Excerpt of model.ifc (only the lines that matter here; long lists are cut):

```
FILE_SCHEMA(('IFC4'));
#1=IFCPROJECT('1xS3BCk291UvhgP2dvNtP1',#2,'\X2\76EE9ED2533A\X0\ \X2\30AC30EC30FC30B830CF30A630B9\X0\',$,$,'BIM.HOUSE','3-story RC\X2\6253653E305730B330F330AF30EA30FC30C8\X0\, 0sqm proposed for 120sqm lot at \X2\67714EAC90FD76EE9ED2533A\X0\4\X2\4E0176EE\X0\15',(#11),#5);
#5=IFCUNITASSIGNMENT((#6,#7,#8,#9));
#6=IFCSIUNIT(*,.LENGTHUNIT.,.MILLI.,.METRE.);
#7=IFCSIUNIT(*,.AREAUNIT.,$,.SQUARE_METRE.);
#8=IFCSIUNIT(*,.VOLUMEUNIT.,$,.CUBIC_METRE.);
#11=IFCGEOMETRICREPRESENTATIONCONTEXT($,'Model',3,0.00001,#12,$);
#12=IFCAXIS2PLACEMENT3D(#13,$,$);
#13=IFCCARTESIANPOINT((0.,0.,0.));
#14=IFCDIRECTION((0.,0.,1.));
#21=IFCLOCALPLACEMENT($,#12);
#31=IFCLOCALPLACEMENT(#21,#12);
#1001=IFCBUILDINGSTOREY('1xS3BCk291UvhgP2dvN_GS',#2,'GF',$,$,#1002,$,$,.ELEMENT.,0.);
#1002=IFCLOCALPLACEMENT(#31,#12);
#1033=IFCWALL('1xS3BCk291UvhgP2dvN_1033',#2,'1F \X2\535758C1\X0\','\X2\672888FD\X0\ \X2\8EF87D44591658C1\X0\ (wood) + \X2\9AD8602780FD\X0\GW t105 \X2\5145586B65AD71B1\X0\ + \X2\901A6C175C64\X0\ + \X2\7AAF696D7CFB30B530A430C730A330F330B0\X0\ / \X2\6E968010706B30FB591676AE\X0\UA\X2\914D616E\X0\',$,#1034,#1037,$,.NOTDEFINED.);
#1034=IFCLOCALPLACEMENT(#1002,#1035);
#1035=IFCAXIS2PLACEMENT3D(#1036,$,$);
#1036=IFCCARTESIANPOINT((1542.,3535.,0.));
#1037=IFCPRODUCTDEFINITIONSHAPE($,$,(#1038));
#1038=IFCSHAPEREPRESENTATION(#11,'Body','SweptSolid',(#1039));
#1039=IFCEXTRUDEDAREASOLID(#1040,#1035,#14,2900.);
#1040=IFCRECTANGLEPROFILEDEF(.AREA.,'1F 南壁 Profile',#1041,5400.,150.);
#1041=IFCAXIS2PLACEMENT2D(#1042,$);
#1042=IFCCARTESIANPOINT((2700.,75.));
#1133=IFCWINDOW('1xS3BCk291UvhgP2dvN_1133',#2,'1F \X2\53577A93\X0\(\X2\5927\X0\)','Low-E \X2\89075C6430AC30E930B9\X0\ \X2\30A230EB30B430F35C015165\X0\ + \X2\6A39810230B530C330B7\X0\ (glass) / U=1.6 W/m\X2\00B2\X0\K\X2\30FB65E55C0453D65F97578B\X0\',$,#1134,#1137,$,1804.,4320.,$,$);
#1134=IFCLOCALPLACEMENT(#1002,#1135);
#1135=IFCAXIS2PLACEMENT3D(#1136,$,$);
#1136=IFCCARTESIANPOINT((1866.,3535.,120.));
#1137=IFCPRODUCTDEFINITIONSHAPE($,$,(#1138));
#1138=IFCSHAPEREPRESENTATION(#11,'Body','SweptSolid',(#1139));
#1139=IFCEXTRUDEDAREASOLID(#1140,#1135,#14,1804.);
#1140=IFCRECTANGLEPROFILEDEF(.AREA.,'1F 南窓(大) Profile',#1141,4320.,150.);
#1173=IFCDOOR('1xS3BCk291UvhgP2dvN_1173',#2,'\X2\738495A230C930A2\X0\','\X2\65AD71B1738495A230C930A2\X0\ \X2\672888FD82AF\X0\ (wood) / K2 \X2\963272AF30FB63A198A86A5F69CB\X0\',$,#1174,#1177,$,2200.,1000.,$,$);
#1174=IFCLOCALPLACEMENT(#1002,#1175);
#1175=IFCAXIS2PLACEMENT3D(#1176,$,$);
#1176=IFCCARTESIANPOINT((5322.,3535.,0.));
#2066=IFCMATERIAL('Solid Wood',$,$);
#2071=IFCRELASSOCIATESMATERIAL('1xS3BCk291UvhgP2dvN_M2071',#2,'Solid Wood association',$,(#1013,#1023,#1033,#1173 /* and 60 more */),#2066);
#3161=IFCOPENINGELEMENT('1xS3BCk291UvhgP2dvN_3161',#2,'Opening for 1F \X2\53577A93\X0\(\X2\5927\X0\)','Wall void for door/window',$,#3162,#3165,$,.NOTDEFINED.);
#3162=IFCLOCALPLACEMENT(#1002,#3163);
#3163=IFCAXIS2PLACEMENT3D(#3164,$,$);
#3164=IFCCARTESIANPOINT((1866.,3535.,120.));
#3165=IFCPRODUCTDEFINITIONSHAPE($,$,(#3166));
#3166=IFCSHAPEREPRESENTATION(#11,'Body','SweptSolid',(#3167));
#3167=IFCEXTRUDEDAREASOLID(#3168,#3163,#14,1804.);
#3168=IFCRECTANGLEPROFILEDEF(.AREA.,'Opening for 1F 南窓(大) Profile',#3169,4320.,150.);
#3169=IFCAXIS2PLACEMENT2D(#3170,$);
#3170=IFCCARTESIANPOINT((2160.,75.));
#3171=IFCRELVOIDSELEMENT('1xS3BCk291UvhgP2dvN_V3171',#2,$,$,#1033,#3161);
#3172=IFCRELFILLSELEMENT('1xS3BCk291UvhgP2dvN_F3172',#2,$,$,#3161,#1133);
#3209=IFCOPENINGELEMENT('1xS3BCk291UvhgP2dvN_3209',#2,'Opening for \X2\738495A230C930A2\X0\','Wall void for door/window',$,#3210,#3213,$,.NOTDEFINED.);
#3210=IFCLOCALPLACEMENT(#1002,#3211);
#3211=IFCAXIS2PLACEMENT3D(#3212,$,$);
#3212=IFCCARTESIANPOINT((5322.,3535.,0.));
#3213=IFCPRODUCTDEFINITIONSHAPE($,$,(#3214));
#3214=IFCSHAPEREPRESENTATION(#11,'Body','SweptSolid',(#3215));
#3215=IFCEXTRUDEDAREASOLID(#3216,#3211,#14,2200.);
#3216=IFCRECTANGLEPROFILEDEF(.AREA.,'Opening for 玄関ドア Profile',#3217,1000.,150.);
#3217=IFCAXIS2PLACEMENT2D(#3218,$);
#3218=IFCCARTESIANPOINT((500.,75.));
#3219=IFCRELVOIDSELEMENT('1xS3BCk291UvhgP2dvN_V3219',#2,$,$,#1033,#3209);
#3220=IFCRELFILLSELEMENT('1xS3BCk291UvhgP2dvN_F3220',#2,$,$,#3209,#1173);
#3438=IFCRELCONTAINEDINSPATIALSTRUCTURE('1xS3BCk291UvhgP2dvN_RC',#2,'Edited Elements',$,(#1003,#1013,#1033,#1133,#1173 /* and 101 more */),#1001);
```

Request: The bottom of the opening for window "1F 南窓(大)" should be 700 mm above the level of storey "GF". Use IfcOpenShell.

```python
import numpy as np
import ifcopenshell
import ifcopenshell.api.geometry
import ifcopenshell.geom
import ifcopenshell.util.element
import ifcopenshell.util.placement
import ifcopenshell.util.shape
import ifcopenshell.util.unit

model = ifcopenshell.open("model.ifc")
unit_scale = ifcopenshell.util.unit.calculate_unit_scale(model)

window = model.by_id(1133)
opening = window.FillsVoids[0].RelatingOpeningElement
storey = ifcopenshell.util.element.get_container(window, ifc_class="IfcBuildingStorey")
level = ifcopenshell.util.placement.get_local_placement(storey.ObjectPlacement)[2, 3]

# The opening's origin need not be at the sill, so measure its lowest point.
shape = ifcopenshell.geom.create_shape(ifcopenshell.geom.settings(), opening)
bottom = ifcopenshell.util.shape.get_shape_bottom_elevation(shape, shape.geometry) / unit_scale
dz = level + 0.7 / unit_scale - bottom

shift = np.array([0.0, 0.0, dz])
# The window is not placed relative to its opening, so move both.
for product in (opening, window):
    matrix = ifcopenshell.util.placement.get_local_placement(product.ObjectPlacement)
    matrix[:3, 3] += shift
    ifcopenshell.api.geometry.edit_object_placement(model, product=product, matrix=matrix, is_si=False)

print(f"moved by {dz * unit_scale:+.3f} m")

model.write("model_updated.ifc")
```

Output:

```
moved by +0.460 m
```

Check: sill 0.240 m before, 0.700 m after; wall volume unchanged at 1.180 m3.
